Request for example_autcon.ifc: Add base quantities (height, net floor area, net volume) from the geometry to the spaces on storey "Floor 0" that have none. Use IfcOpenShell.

First a look at what the model holds.

```python
import ifcopenshell
import ifcopenshell.util.element
import ifcopenshell.util.unit

model = ifcopenshell.open("example_autcon.ifc")
print(model.schema)
for unit_type in ("LENGTHUNIT", "AREAUNIT", "VOLUMEUNIT"):
    print(unit_type, ifcopenshell.util.unit.calculate_unit_scale(model, unit_type))
storey = next(s for s in model.by_type("IfcBuildingStorey") if s.Name == "Floor 0")
spaces = [e for e in ifcopenshell.util.element.get_decomposition(storey) if e.is_a("IfcSpace")]
for e in sorted(spaces, key=lambda e: e.id()):
    print(e.id(), e.is_a(), e.Name, list(ifcopenshell.util.element.get_psets(e, qtos_only=True)), sep=" | ")
```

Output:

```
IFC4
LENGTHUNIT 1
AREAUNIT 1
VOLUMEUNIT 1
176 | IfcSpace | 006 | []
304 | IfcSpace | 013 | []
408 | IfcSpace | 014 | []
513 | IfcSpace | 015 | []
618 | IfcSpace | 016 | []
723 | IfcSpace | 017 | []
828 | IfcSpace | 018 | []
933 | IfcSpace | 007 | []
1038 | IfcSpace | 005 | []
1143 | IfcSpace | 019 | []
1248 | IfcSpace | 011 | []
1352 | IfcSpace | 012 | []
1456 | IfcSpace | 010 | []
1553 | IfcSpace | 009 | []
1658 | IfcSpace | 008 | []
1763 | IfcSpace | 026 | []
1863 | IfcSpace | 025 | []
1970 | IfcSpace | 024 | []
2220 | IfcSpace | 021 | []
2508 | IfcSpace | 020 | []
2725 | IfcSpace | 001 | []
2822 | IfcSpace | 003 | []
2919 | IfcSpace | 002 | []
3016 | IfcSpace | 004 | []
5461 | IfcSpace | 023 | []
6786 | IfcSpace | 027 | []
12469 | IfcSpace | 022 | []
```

```python
import ifcopenshell
import ifcopenshell.api.pset
import ifcopenshell.geom
import ifcopenshell.util.element
import ifcopenshell.util.shape
import ifcopenshell.util.unit

model = ifcopenshell.open("example_autcon.ifc")
unit_scale = ifcopenshell.util.unit.calculate_unit_scale(model)
area_scale = ifcopenshell.util.unit.calculate_unit_scale(model, "AREAUNIT")
volume_scale = ifcopenshell.util.unit.calculate_unit_scale(model, "VOLUMEUNIT")
settings = ifcopenshell.geom.settings()

storey = next(s for s in model.by_type("IfcBuildingStorey") if s.Name == "Floor 0")
spaces = [e for e in ifcopenshell.util.element.get_decomposition(storey) if e.is_a("IfcSpace")]

for e in sorted(spaces, key=lambda e: e.id()):
    if ifcopenshell.util.element.get_psets(e, qtos_only=True, should_inherit=False):
        continue
    # Geometry comes back in metres, in the element's own axes.
    shape = ifcopenshell.geom.create_shape(settings, e)
    values = {
        "Height": ifcopenshell.util.shape.get_z(shape.geometry) / unit_scale,
        "NetFloorArea": ifcopenshell.util.shape.get_footprint_area(shape.geometry) / area_scale,
        "NetVolume": ifcopenshell.util.shape.get_volume(shape.geometry) / volume_scale,
    }
    qto = ifcopenshell.api.pset.add_qto(model, product=e, name="Qto_SpaceBaseQuantities")
    ifcopenshell.api.pset.edit_qto(model, qto=qto, properties=values)
    print(e.id(), {k: round(v, 3) for k, v in values.items()})

model.write("example_autcon_v2.ifc")
```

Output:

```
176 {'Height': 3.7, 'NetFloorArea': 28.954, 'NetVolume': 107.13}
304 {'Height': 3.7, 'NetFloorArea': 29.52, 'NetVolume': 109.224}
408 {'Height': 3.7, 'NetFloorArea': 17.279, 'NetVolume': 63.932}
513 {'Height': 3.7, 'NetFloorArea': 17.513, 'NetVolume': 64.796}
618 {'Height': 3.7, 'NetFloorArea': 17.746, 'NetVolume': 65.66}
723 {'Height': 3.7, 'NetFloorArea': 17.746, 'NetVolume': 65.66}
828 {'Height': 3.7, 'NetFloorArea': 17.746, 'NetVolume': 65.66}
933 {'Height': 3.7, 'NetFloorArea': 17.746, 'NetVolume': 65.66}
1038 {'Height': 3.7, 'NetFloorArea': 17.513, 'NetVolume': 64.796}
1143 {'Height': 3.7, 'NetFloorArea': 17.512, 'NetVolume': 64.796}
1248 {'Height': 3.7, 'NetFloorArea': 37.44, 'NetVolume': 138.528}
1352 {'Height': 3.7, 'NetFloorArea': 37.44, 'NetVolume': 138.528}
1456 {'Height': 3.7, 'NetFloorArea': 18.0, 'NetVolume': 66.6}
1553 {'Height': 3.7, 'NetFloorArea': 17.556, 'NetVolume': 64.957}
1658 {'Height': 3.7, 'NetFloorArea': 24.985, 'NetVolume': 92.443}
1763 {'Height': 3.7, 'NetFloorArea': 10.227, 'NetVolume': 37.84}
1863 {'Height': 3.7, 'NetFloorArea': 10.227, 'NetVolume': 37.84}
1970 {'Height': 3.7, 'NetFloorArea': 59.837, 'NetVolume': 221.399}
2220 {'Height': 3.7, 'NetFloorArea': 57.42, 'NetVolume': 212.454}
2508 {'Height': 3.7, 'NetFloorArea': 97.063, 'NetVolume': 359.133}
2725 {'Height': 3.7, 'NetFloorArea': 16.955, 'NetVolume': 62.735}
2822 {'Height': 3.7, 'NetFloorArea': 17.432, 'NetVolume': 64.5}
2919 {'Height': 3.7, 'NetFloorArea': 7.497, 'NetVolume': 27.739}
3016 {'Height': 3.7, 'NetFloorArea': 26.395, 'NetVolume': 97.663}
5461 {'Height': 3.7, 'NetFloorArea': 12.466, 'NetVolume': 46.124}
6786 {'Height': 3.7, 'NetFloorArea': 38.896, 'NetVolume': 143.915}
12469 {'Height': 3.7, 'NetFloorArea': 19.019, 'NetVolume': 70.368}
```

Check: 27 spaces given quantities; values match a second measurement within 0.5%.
